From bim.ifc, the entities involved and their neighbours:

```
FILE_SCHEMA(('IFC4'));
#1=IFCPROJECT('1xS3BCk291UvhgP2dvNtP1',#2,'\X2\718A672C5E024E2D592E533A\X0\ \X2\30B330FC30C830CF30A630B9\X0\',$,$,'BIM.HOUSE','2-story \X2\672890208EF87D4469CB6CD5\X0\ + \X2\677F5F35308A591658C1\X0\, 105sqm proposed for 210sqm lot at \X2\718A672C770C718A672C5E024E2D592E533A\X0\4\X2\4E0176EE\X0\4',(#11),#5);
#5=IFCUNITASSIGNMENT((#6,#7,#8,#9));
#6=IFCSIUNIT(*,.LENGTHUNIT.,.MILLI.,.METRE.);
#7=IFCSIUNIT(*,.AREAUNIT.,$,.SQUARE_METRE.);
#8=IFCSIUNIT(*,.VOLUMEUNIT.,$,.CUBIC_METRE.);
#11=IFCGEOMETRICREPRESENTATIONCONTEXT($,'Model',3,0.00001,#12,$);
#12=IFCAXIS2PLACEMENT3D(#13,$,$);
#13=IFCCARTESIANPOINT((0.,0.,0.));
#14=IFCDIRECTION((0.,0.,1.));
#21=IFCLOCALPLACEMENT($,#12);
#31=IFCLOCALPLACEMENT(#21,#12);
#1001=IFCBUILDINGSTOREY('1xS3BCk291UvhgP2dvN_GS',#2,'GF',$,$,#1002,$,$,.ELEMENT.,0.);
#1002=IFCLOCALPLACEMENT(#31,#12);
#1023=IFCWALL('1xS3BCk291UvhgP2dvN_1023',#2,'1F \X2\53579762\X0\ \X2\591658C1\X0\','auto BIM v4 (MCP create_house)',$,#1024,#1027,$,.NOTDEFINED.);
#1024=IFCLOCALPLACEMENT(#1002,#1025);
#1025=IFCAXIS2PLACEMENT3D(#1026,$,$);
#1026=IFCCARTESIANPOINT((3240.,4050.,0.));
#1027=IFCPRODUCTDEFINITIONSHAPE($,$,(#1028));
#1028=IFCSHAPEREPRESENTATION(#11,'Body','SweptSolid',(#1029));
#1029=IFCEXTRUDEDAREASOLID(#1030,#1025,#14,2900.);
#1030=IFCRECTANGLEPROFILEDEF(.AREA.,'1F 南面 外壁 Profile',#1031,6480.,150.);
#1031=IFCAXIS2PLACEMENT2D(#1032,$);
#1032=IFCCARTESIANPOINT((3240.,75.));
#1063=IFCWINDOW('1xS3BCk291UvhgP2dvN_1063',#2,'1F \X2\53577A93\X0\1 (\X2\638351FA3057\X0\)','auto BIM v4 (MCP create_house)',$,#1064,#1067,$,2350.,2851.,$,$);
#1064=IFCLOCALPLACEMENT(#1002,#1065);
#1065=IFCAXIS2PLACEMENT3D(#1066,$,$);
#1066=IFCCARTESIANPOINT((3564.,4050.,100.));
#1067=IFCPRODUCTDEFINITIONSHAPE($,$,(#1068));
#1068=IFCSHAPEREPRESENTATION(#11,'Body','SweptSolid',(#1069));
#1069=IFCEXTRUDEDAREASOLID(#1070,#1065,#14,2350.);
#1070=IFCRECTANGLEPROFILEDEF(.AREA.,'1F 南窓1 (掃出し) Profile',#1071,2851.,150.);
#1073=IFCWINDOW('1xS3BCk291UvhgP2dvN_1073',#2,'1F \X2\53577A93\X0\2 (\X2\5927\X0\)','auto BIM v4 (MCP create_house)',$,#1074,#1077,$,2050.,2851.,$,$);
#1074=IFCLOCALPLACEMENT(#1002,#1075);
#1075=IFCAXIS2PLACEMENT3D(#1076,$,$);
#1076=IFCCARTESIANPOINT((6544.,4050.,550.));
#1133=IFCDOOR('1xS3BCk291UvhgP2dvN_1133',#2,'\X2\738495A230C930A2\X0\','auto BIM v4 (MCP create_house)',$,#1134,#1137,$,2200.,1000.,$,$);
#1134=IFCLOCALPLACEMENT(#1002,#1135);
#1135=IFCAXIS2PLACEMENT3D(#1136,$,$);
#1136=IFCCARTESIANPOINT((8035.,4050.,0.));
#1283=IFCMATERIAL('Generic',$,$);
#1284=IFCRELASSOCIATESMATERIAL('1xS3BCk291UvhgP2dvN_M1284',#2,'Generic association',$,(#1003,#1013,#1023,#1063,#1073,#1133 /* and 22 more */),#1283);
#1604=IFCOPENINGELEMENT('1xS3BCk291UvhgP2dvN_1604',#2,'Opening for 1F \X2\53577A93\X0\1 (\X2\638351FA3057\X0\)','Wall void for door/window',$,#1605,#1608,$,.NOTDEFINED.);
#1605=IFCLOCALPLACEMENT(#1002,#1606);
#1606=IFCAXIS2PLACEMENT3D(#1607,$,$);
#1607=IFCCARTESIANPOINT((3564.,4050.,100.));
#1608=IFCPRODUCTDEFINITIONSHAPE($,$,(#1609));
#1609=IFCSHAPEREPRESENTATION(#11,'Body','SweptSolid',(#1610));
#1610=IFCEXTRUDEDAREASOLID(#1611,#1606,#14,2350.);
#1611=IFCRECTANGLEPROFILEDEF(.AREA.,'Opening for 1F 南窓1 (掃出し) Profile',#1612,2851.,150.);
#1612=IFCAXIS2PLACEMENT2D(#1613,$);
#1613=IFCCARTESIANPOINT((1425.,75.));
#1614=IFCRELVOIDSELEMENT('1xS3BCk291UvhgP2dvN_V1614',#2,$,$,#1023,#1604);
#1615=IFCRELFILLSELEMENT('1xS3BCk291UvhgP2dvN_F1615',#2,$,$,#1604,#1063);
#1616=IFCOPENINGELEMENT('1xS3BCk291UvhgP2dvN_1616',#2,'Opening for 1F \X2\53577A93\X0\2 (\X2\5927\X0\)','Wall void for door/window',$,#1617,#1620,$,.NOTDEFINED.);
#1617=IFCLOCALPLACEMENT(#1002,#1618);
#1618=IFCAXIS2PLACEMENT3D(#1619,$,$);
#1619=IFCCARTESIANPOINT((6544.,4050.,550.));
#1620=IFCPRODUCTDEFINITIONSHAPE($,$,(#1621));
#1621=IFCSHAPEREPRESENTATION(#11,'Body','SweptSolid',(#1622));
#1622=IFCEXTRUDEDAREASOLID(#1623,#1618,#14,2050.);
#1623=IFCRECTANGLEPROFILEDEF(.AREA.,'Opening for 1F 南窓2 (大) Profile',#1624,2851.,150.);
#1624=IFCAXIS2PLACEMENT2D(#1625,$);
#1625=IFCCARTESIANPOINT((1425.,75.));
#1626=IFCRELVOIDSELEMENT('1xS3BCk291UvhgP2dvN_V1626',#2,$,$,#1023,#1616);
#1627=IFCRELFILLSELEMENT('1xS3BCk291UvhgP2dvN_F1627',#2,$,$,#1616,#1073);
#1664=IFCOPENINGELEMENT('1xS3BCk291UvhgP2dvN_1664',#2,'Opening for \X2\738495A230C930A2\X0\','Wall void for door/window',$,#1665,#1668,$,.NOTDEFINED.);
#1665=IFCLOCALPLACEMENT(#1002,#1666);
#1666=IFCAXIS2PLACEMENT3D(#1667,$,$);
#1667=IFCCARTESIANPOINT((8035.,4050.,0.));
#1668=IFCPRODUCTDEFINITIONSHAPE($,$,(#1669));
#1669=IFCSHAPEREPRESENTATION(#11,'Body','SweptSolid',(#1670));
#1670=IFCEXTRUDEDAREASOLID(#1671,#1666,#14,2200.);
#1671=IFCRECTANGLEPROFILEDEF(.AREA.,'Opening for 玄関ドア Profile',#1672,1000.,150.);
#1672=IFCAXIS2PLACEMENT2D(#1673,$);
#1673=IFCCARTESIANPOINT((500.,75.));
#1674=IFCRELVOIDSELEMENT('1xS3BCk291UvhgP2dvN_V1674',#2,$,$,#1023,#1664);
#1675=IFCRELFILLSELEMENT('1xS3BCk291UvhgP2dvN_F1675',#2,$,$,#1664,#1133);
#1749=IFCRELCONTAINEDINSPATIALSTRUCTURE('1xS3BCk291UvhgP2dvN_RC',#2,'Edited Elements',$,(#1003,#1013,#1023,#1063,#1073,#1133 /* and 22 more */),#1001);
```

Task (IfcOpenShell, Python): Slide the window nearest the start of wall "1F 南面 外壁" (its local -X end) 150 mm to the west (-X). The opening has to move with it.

```python
import ifcopenshell
import ifcopenshell.api.geometry
import ifcopenshell.util.placement

model = ifcopenshell.open("bim.ifc")

window = model.by_guid("1xS3BCk291UvhgP2dvN_1063")
opening = window.FillsVoids[0].RelatingOpeningElement
wall = opening.VoidsElements[0].RelatingBuildingElement

wall_matrix = ifcopenshell.util.placement.get_local_placement(wall.ObjectPlacement)
shift = wall_matrix[:3, 0] * -150.0
before = ifcopenshell.util.placement.get_local_placement(window.ObjectPlacement)[:3, 3].copy()

# The window is not placed relative to its opening, so move both.
for product in (opening, window):
    matrix = ifcopenshell.util.placement.get_local_placement(product.ObjectPlacement)
    matrix[:3, 3] += shift
    ifcopenshell.api.geometry.edit_object_placement(model, product=product, matrix=matrix, is_si=False)

after = ifcopenshell.util.placement.get_local_placement(window.ObjectPlacement)[:3, 3]
print("window moved by", (after - before).round(3) + 0.0)

model.write("bim_v2.ifc")
```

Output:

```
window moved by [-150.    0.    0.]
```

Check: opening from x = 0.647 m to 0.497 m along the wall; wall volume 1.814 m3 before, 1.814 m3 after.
